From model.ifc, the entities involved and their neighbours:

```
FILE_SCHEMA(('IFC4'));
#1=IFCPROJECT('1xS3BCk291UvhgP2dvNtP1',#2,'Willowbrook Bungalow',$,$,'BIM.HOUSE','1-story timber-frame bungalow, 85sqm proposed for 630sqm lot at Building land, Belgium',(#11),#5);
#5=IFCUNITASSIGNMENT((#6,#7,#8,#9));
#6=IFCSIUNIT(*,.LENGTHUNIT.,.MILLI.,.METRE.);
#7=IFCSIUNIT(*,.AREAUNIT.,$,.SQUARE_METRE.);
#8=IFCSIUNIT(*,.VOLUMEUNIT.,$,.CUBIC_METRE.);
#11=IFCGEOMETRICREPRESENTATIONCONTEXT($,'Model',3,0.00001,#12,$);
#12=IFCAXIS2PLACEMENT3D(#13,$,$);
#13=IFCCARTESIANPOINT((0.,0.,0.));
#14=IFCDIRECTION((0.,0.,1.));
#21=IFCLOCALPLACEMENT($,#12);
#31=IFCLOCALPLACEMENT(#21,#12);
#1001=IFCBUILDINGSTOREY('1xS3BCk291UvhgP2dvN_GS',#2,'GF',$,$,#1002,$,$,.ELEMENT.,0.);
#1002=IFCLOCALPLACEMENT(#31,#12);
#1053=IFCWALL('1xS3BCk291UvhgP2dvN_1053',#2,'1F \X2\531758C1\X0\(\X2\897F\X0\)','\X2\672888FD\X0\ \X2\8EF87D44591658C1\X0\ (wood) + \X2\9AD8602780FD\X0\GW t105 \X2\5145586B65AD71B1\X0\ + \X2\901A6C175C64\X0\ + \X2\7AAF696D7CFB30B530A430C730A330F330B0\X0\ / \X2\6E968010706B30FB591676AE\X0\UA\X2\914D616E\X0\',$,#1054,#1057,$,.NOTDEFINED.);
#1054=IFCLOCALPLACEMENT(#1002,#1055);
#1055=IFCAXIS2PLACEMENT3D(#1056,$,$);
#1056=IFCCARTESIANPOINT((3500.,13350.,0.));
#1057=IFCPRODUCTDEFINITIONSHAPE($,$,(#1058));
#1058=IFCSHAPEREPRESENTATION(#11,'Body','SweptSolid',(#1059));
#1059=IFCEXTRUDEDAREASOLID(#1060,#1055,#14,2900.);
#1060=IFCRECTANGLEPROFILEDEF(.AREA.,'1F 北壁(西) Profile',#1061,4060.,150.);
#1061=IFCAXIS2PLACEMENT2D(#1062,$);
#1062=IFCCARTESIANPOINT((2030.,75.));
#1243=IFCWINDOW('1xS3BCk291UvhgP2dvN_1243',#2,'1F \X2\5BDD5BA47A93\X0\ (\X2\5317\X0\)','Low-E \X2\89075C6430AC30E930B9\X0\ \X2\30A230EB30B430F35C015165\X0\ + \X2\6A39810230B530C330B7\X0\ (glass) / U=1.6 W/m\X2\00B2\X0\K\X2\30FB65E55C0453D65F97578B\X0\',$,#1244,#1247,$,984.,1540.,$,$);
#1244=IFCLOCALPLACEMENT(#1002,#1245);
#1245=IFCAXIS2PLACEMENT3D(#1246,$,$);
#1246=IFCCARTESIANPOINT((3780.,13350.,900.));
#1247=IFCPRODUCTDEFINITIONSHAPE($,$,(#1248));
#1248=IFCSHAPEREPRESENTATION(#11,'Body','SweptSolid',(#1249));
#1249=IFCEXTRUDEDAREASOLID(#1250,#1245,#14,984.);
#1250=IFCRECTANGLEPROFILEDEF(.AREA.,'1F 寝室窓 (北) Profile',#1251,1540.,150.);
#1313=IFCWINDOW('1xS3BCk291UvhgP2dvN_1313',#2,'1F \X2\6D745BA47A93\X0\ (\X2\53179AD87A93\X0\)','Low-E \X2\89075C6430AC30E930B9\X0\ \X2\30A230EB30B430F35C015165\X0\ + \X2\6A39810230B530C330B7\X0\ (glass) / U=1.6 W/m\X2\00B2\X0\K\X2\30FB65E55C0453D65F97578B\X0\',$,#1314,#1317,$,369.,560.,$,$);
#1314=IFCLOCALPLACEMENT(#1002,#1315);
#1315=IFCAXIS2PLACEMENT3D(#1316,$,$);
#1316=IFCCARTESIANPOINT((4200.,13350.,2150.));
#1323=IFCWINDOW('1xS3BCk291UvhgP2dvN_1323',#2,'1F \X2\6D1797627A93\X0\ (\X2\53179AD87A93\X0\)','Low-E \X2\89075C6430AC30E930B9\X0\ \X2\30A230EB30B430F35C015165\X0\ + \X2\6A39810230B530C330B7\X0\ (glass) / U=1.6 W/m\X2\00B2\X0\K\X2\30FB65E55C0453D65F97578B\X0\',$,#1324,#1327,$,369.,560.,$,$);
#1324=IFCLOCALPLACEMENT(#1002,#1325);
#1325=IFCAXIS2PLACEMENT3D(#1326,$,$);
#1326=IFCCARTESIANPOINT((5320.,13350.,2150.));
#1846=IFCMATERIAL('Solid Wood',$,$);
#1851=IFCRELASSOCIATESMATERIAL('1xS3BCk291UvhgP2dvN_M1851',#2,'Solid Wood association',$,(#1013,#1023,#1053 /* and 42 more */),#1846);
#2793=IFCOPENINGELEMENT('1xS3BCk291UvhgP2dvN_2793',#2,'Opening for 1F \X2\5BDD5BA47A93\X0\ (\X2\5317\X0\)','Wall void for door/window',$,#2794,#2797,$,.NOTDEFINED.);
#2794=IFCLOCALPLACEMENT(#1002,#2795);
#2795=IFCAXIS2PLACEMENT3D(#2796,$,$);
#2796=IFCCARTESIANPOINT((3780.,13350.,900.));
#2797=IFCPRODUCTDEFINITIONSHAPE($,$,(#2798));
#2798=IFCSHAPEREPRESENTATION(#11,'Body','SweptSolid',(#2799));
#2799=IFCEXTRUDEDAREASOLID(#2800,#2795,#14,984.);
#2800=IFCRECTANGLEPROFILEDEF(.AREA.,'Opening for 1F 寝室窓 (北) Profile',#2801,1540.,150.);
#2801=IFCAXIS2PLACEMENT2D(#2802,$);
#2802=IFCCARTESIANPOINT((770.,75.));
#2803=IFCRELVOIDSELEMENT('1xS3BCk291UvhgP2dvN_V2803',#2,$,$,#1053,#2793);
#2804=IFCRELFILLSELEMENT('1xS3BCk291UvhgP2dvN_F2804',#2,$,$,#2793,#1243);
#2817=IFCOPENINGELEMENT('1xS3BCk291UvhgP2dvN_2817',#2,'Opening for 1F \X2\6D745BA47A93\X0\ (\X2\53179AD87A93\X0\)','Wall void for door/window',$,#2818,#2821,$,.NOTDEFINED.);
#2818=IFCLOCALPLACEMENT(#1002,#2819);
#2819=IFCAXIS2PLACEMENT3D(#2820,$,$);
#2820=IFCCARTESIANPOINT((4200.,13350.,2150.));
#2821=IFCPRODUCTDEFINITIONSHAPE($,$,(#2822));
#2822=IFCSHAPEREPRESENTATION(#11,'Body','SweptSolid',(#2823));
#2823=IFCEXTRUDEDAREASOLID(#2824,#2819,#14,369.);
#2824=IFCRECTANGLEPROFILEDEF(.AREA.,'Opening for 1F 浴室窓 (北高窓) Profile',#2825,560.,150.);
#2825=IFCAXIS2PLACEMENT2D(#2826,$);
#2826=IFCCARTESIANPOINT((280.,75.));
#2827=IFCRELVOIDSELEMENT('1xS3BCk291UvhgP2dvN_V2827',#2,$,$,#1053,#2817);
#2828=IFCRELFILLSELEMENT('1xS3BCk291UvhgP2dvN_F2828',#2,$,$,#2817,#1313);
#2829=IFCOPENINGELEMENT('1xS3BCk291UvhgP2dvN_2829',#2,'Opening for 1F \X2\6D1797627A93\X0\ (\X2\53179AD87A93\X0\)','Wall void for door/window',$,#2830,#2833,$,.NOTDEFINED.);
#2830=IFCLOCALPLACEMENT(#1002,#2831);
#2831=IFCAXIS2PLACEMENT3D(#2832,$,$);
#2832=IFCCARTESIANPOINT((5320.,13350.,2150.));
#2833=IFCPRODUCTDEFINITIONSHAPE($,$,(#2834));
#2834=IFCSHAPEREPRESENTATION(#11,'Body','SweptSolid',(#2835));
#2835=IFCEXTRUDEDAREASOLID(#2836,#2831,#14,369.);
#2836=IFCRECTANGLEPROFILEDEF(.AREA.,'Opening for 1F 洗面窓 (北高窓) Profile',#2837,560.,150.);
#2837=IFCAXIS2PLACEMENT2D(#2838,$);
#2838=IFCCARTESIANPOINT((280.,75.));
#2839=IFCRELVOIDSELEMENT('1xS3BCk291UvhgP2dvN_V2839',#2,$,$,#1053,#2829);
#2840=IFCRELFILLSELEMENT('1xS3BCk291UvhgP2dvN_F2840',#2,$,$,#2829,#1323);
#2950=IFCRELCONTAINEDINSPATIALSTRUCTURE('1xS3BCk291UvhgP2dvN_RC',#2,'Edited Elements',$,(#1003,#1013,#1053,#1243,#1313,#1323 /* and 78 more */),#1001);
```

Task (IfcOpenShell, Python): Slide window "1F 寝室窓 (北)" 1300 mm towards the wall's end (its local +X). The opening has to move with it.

```python
import ifcopenshell
import ifcopenshell.api.geometry
import ifcopenshell.util.placement
import ifcopenshell.util.unit

model = ifcopenshell.open("model.ifc")
unit_scale = ifcopenshell.util.unit.calculate_unit_scale(model)

window = model.by_id(1243)
opening = window.FillsVoids[0].RelatingOpeningElement
wall = opening.VoidsElements[0].RelatingBuildingElement

wall_matrix = ifcopenshell.util.placement.get_local_placement(wall.ObjectPlacement)
shift = wall_matrix[:3, 0] * 1.3 / unit_scale
before = ifcopenshell.util.placement.get_local_placement(window.ObjectPlacement)[:3, 3].copy()

# The window is not placed relative to its opening, so move both.
for product in (opening, window):
    matrix = ifcopenshell.util.placement.get_local_placement(product.ObjectPlacement)
    matrix[:3, 3] += shift
    ifcopenshell.api.geometry.edit_object_placement(model, product=product, matrix=matrix, is_si=False)

after = ifcopenshell.util.placement.get_local_placement(window.ObjectPlacement)[:3, 3]
print("window moved by", (after - before).round(3) + 0.0)

model.write("model_rev.ifc")
```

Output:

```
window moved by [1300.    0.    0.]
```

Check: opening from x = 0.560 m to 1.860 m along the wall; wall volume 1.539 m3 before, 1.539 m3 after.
